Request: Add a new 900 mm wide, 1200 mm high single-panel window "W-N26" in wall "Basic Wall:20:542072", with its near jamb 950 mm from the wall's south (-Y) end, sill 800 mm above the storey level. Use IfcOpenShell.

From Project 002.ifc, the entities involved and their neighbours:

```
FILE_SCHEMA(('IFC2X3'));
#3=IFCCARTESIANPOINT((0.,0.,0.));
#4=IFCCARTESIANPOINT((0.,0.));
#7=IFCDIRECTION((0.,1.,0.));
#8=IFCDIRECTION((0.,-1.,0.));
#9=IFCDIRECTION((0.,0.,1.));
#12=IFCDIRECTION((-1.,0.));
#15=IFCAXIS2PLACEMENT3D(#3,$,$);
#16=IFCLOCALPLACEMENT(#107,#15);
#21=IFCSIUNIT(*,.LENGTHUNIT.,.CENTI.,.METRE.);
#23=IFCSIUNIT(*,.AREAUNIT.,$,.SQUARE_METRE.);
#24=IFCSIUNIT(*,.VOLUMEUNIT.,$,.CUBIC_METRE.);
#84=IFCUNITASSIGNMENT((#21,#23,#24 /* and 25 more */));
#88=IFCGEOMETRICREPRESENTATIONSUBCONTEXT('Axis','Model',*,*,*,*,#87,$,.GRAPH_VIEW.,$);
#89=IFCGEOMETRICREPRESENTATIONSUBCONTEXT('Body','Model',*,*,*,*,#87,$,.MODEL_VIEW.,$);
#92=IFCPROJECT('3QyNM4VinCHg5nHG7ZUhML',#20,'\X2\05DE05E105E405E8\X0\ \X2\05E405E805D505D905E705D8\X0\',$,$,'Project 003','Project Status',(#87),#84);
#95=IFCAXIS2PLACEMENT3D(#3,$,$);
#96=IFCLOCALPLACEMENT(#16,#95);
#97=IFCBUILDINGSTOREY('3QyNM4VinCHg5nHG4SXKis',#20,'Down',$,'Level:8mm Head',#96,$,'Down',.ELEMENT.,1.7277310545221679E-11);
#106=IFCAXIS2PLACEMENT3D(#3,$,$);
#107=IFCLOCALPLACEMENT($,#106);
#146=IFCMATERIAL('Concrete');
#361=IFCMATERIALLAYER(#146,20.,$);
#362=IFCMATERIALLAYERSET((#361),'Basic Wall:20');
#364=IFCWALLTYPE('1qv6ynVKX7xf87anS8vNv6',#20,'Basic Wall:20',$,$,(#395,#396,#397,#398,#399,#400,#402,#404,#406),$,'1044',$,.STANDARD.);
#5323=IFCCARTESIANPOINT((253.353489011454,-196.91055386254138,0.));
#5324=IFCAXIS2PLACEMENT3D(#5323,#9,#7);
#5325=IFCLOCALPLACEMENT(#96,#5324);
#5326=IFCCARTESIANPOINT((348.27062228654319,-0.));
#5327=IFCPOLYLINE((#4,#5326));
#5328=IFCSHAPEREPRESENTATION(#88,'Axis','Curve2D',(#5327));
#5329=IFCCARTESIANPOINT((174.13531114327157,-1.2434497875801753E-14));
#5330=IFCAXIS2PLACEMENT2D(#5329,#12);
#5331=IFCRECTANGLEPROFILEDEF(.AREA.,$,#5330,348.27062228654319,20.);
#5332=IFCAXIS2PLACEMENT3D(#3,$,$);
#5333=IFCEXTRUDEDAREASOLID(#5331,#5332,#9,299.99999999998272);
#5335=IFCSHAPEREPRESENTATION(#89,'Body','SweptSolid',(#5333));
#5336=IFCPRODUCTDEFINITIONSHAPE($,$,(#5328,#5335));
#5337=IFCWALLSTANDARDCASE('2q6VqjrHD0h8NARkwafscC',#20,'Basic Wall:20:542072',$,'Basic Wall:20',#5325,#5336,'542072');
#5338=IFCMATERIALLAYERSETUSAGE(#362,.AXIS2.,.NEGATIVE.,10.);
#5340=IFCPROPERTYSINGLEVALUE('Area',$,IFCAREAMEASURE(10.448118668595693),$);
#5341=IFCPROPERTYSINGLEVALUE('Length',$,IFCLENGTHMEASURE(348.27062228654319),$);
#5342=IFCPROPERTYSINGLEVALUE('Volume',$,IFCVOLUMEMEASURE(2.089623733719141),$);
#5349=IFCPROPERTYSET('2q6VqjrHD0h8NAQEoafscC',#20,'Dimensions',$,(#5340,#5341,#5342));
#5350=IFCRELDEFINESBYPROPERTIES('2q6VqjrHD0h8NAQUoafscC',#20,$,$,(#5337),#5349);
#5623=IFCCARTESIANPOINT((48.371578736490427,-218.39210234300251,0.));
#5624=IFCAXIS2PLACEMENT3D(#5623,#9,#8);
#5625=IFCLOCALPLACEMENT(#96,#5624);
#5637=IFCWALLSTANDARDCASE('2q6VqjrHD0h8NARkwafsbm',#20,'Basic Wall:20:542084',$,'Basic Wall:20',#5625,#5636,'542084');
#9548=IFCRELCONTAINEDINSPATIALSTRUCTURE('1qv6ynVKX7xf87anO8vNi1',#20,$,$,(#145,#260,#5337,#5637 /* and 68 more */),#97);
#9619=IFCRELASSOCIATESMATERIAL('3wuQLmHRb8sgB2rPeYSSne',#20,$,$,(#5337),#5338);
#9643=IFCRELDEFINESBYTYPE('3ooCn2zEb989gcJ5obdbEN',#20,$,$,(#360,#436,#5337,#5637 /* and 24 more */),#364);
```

```python
import numpy as np
import ifcopenshell
import ifcopenshell.api.feature
import ifcopenshell.api.geometry
import ifcopenshell.api.pset
import ifcopenshell.api.root
import ifcopenshell.api.spatial
import ifcopenshell.api.type
import ifcopenshell.geom
import ifcopenshell.util.element
import ifcopenshell.util.placement
import ifcopenshell.util.representation
import ifcopenshell.util.shape
import ifcopenshell.util.unit

model = ifcopenshell.open("Project 002.ifc")
unit_scale = ifcopenshell.util.unit.calculate_unit_scale(model)
area_scale = ifcopenshell.util.unit.calculate_unit_scale(model, "AREAUNIT")
volume_scale = ifcopenshell.util.unit.calculate_unit_scale(model, "VOLUMEUNIT")
settings = ifcopenshell.geom.settings()


def volume(element):
    """Net volume in cubic metres, openings subtracted."""
    shape = ifcopenshell.geom.create_shape(settings, element)
    return ifcopenshell.util.shape.get_volume(shape.geometry)


wall = model.by_guid("2q6VqjrHD0h8NARkwafscC")
storey = ifcopenshell.util.element.get_container(wall, ifc_class="IfcBuildingStorey")
context = ifcopenshell.util.representation.get_context(model, "Model", "Body", "MODEL_VIEW")
before = volume(wall)

width, height, from_end, sill = 0.9, 1.2, 0.95, 0.8  # metres

# The wall runs along its own X axis, and the end named is its -X end.
wall_shape = ifcopenshell.geom.create_shape(settings, wall)
x, y, z = ifcopenshell.util.shape.get_vertices(wall_shape.geometry).T
start = x.min() + from_end
face, thickness = float(y.min()), float(y.max() - y.min())
wall_matrix = ifcopenshell.util.placement.get_local_placement(wall.ObjectPlacement)
level = ifcopenshell.util.placement.get_local_placement(storey.ObjectPlacement)[2, 3]


def in_wall(x, y):
    """Placement at x, y metres in the wall's axes, at sill height."""
    matrix = wall_matrix.copy()
    matrix[:, 3] = wall_matrix @ np.array([x / unit_scale, y / unit_scale, 0.0, 1.0])
    matrix[2, 3] = level + sill / unit_scale
    return matrix


# Opening: a box that overshoots both wall faces by 50 mm.
opening = ifcopenshell.api.root.create_entity(model, ifc_class="IfcOpeningElement")
box = ifcopenshell.api.geometry.add_wall_representation(
    model, context=context, length=width, height=height, thickness=thickness + 0.1
)
ifcopenshell.api.geometry.assign_representation(model, product=opening, representation=box)
ifcopenshell.api.geometry.edit_object_placement(model, product=opening, matrix=in_wall(start, face - 0.05), is_si=False)
ifcopenshell.api.feature.add_feature(model, feature=opening, element=wall)

window = ifcopenshell.api.root.create_entity(model, ifc_class="IfcWindow", name="W-N26")
window.OverallWidth, window.OverallHeight = width / unit_scale, height / unit_scale
body = ifcopenshell.api.geometry.add_window_representation(
    model,
    context=context,
    overall_width=window.OverallWidth,
    overall_height=window.OverallHeight,
    partition_type="SINGLE_PANEL",
)
ifcopenshell.api.geometry.assign_representation(model, product=window, representation=body)
ifcopenshell.api.spatial.assign_container(model, products=[window], relating_structure=storey)
fills = ifcopenshell.api.feature.add_filling(model, opening=opening, element=window)
fills.OwnerHistory = window.OwnerHistory  # required in IFC2X3

# IFC2X3 keeps the operation on the window style.
style = ifcopenshell.api.root.create_entity(model, ifc_class="IfcWindowStyle", name="W-N26")
style.OperationType, style.ConstructionType = "SINGLE_PANEL", "NOTDEFINED"
style.ParameterTakesPrecedence = style.Sizeable = False
ifcopenshell.api.type.assign_type(model, related_objects=[window], relating_type=style)

# Centre the window in the wall's thickness.
ifcopenshell.api.geometry.edit_object_placement(model, product=window, matrix=in_wall(start, face), is_si=False)
window_shape = ifcopenshell.geom.create_shape(settings, window)
depth = ifcopenshell.util.shape.get_vertices(window_shape.geometry)[:, 1]
offset = face + thickness / 2 - (depth.min() + depth.max()) / 2
ifcopenshell.api.geometry.edit_object_placement(model, product=window, matrix=in_wall(start, offset), is_si=False)

after = volume(wall)

# Update the wall's stored quantities.
pset = model.by_id(ifcopenshell.util.element.get_pset(wall, "Dimensions", should_inherit=False)["id"])
ifcopenshell.api.pset.edit_pset(model, pset=pset, properties={
    "Area": model.create_entity("IfcAreaMeasure", after / thickness / area_scale),
    "Volume": model.create_entity("IfcVolumeMeasure", after / volume_scale),
})

print(f"wall volume {before:.3f} -> {after:.3f} m3")

model.write("Project 002_v2.ifc")
```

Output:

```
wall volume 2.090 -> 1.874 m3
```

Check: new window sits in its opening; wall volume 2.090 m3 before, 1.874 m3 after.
